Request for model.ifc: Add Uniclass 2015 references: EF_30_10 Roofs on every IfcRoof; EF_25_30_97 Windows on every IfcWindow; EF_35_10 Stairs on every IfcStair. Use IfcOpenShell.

First a look at what the model holds.

```python
import ifcopenshell

model = ifcopenshell.open("model.ifc")
print(model.schema)
print("classifications:", [c.Name for c in model.by_type("IfcClassification")])
for ifc_class in ("IfcDoor", "IfcRoof", "IfcStair", "IfcWall", "IfcWindow"):
    print(ifc_class, len(model.by_type(ifc_class)))
```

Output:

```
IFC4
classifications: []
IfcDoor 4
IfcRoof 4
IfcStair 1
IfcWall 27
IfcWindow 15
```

```python
import ifcopenshell
import ifcopenshell.api.classification

model = ifcopenshell.open("model.ifc")

system = ifcopenshell.api.classification.add_classification(model, classification="Uniclass 2015")

codes = {
    "IfcRoof": ("EF_30_10", "Roofs"),
    "IfcWindow": ("EF_25_30_97", "Windows"),
    "IfcStair": ("EF_35_10", "Stairs"),
}
for ifc_class, (code, name) in codes.items():
    products = model.by_type(ifc_class)
    ifcopenshell.api.classification.add_reference(
        model, products=products, classification=system, identification=code, name=name
    )
    print(code, len(products))

model.write("model_v2.ifc")
```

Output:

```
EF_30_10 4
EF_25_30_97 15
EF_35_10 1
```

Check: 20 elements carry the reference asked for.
